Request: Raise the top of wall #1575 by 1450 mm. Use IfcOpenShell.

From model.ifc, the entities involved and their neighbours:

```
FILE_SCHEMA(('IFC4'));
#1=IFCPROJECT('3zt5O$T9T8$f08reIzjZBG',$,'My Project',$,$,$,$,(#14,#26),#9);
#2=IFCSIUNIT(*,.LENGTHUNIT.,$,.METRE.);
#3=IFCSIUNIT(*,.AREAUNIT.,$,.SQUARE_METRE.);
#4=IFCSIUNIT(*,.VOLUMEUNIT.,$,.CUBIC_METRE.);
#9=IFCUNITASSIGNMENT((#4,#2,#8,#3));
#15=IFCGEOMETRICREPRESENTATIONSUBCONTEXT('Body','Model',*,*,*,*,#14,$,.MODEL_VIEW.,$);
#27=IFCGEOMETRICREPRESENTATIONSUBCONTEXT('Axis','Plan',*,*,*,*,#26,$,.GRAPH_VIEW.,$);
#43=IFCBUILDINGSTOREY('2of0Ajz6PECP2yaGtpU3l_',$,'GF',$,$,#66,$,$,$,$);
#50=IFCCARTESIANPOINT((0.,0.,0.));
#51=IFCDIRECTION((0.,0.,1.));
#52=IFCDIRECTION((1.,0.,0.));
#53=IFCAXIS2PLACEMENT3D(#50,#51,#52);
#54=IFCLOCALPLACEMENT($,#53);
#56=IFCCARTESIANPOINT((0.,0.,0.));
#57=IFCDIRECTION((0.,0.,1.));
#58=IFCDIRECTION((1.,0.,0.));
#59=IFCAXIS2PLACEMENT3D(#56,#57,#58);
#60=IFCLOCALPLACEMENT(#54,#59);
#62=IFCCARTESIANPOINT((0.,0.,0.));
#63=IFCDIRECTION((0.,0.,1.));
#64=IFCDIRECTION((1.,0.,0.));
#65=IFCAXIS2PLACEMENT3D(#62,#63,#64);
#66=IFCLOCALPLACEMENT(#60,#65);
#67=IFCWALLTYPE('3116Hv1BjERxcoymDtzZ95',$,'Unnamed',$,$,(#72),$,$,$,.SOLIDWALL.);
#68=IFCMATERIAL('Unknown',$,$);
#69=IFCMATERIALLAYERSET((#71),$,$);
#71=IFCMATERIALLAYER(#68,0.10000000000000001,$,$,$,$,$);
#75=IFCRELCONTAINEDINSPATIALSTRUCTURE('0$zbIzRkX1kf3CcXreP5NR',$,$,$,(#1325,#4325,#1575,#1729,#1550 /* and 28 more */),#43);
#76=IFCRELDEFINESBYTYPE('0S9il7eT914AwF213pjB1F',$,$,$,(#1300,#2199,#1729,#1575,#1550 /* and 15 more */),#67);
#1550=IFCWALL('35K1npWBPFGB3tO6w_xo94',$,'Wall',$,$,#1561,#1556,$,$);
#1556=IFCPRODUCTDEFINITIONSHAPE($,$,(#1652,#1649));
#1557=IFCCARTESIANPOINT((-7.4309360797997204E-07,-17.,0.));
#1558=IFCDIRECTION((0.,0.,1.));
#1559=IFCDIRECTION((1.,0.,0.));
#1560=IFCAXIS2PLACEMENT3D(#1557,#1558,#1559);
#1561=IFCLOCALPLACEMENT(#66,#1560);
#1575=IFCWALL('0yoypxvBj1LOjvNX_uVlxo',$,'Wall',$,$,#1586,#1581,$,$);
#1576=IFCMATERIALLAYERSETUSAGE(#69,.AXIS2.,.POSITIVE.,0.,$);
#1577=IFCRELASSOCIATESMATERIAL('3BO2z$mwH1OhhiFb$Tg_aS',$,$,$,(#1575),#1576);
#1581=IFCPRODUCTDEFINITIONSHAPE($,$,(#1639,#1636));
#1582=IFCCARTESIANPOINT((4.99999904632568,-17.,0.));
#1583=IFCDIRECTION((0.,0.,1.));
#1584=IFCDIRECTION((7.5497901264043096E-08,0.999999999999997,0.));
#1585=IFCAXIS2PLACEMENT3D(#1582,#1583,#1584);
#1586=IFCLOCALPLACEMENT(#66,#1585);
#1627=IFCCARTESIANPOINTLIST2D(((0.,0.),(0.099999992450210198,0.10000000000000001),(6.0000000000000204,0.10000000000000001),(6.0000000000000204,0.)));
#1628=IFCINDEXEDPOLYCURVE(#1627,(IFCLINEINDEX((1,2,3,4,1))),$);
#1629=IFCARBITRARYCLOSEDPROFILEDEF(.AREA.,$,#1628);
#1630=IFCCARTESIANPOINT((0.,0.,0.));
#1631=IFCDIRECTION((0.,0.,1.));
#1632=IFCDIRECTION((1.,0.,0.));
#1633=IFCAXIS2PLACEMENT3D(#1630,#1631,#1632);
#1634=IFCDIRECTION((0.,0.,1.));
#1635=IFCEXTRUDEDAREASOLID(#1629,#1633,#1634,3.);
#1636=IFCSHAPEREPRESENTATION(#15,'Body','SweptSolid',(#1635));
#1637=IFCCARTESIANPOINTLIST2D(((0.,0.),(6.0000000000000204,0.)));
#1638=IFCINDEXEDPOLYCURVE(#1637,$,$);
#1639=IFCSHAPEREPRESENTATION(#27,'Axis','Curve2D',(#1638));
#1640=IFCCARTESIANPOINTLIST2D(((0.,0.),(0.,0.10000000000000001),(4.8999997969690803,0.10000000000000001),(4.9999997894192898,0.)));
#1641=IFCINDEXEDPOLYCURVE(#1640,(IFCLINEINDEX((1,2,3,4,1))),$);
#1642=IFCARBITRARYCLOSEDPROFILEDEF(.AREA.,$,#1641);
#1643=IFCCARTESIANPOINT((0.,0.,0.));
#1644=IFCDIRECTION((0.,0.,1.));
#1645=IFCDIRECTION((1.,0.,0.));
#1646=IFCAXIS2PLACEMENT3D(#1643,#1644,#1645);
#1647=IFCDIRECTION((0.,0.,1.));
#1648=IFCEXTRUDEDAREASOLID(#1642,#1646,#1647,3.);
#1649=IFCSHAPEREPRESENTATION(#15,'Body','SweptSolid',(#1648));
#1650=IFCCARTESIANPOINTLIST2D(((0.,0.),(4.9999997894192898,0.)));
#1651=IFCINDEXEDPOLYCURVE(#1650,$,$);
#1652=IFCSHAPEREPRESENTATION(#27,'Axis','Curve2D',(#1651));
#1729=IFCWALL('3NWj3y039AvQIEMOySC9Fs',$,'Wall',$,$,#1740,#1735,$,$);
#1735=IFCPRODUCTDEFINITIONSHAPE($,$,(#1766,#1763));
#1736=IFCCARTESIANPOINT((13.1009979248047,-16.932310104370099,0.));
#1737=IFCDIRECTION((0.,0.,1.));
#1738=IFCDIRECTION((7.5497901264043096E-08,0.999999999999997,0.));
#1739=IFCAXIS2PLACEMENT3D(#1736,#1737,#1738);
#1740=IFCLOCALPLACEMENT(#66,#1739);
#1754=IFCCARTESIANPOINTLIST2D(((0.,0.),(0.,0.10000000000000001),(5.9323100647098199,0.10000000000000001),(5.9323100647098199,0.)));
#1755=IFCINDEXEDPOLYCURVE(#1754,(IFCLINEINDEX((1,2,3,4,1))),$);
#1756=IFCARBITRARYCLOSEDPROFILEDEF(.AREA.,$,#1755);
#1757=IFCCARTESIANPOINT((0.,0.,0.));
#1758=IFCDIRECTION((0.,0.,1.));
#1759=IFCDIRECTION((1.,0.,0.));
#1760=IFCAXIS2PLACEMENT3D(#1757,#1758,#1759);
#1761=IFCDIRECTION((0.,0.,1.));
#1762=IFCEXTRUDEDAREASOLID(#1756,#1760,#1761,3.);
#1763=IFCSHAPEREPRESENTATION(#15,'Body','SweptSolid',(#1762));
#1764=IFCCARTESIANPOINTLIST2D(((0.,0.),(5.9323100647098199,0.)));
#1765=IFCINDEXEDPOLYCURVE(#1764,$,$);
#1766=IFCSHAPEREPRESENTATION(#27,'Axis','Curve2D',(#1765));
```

```python
import ifcopenshell
import ifcopenshell.geom
import ifcopenshell.util.representation
import ifcopenshell.util.shape

model = ifcopenshell.open("model.ifc")
settings = ifcopenshell.geom.settings()


def volume(element):
    """Net volume in cubic metres, openings subtracted."""
    shape = ifcopenshell.geom.create_shape(settings, element)
    return ifcopenshell.util.shape.get_volume(shape.geometry)


wall = model.by_guid("0yoypxvBj1LOjvNX_uVlxo")
before = volume(wall)

body = ifcopenshell.util.representation.get_representation(wall, "Model", "Body")
solid = body.Items[0]
old_height = solid.Depth
solid.Depth += 1.45
after = volume(wall)

print(f"height {old_height:g} -> {solid.Depth:g}, volume {before:.3f} -> {after:.3f} m3")

model.write("model_v2.ifc")
```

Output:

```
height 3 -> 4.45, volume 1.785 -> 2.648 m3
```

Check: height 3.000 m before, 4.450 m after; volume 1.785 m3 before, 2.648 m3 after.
